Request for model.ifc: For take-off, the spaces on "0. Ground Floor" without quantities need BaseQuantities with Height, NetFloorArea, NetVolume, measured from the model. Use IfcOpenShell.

First a look at what the model holds.

```python
import ifcopenshell
import ifcopenshell.util.element
import ifcopenshell.util.unit

model = ifcopenshell.open("model.ifc")
print(model.schema)
for unit_type in ("LENGTHUNIT", "AREAUNIT", "VOLUMEUNIT"):
    print(unit_type, ifcopenshell.util.unit.calculate_unit_scale(model, unit_type))
storey = next(s for s in model.by_type("IfcBuildingStorey") if s.Name == "0. Ground Floor")
spaces = [e for e in ifcopenshell.util.element.get_decomposition(storey) if e.is_a("IfcSpace")]
for e in sorted(spaces, key=lambda e: e.id()):
    print(e.id(), e.is_a(), e.Name, list(ifcopenshell.util.element.get_psets(e, qtos_only=True)), sep=" | ")
```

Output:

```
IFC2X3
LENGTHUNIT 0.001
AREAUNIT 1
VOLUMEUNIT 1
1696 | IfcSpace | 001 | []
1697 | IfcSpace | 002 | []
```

```python
import ifcopenshell
import ifcopenshell.api.pset
import ifcopenshell.geom
import ifcopenshell.util.element
import ifcopenshell.util.shape
import ifcopenshell.util.unit

model = ifcopenshell.open("model.ifc")
unit_scale = ifcopenshell.util.unit.calculate_unit_scale(model)
area_scale = ifcopenshell.util.unit.calculate_unit_scale(model, "AREAUNIT")
volume_scale = ifcopenshell.util.unit.calculate_unit_scale(model, "VOLUMEUNIT")
settings = ifcopenshell.geom.settings()

storey = next(s for s in model.by_type("IfcBuildingStorey") if s.Name == "0. Ground Floor")
spaces = [e for e in ifcopenshell.util.element.get_decomposition(storey) if e.is_a("IfcSpace")]

for e in sorted(spaces, key=lambda e: e.id()):
    if ifcopenshell.util.element.get_psets(e, qtos_only=True, should_inherit=False):
        continue
    # Geometry comes back in metres, in the element's own axes.
    shape = ifcopenshell.geom.create_shape(settings, e)
    values = {
        "Height": ifcopenshell.util.shape.get_z(shape.geometry) / unit_scale,
        "NetFloorArea": ifcopenshell.util.shape.get_footprint_area(shape.geometry) / area_scale,
        "NetVolume": ifcopenshell.util.shape.get_volume(shape.geometry) / volume_scale,
    }
    qto = ifcopenshell.api.pset.add_qto(model, product=e, name="BaseQuantities")
    ifcopenshell.api.pset.edit_qto(model, qto=qto, properties=values)
    print(e.id(), {k: round(v, 3) for k, v in values.items()})

model.write("model_v2.ifc")
```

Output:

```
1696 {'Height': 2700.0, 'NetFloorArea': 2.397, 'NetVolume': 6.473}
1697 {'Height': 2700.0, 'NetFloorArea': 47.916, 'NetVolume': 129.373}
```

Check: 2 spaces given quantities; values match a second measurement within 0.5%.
